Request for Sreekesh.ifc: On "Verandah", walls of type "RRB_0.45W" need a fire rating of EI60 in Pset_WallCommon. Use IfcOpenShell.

First a look at what the model holds.

```python
import ifcopenshell
import ifcopenshell.util.element

model = ifcopenshell.open("Sreekesh.ifc")
print(model.schema)
storey = next(s for s in model.by_type("IfcBuildingStorey") if s.Name == "Verandah")
walls = [e for e in ifcopenshell.util.element.get_decomposition(storey) if e.is_a("IfcWall")]
seen = {}
for e in walls:
    element_type = ifcopenshell.util.element.get_type(e)
    key = (element_type.Name if element_type != e and element_type else None, ifcopenshell.util.element.get_pset(e, "Pset_WallCommon", "FireRating"))
    seen[key] = seen.get(key, 0) + 1
for (name, value), count in sorted(seen.items(), key=str):
    print(count, "x", name, "|", value)
```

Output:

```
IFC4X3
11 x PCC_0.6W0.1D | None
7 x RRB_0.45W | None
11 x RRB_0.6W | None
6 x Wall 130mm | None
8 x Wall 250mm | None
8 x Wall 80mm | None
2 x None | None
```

```python
import ifcopenshell
import ifcopenshell.api.pset
import ifcopenshell.util.element

model = ifcopenshell.open("Sreekesh.ifc")

storey = next(s for s in model.by_type("IfcBuildingStorey") if s.Name == "Verandah")
walls = [e for e in ifcopenshell.util.element.get_decomposition(storey) if e.is_a("IfcWall")]

count = 0
for e in walls:
    element_type = ifcopenshell.util.element.get_type(e)
    if element_type in (None, e) or element_type.Name != "RRB_0.45W":
        continue
    # add_pset returns the element's existing set when there is one.
    pset = ifcopenshell.api.pset.add_pset(model, product=e, name="Pset_WallCommon")
    ifcopenshell.api.pset.edit_pset(model, pset=pset, properties={"FireRating": "EI60"})
    count += 1

print(count, "walls updated")

model.write("Sreekesh_edited.ifc")
```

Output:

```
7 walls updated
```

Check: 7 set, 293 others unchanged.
